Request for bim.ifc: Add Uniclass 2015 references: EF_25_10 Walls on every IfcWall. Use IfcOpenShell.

First a look at what the model holds.

```python
import ifcopenshell

model = ifcopenshell.open("bim.ifc")
print(model.schema)
print("classifications:", [c.Name for c in model.by_type("IfcClassification")])
for ifc_class in ("IfcDoor", "IfcRoof", "IfcStair", "IfcWall", "IfcWindow"):
    print(ifc_class, len(model.by_type(ifc_class)))
```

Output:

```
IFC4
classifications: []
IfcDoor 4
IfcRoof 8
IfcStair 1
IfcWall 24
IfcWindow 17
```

```python
import ifcopenshell
import ifcopenshell.api.classification

model = ifcopenshell.open("bim.ifc")

system = ifcopenshell.api.classification.add_classification(model, classification="Uniclass 2015")

codes = {
    "IfcWall": ("EF_25_10", "Walls"),
}
for ifc_class, (code, name) in codes.items():
    products = model.by_type(ifc_class)
    ifcopenshell.api.classification.add_reference(
        model, products=products, classification=system, identification=code, name=name
    )
    print(code, len(products))

model.write("bim_edited.ifc")
```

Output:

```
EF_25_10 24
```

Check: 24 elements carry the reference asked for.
